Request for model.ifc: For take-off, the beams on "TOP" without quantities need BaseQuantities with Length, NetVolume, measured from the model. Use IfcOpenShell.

First a look at what the model holds.

```python
import ifcopenshell
import ifcopenshell.util.element
import ifcopenshell.util.unit

model = ifcopenshell.open("model.ifc")
print(model.schema)
for unit_type in ("LENGTHUNIT", "AREAUNIT", "VOLUMEUNIT"):
    print(unit_type, ifcopenshell.util.unit.calculate_unit_scale(model, unit_type))
storey = next(s for s in model.by_type("IfcBuildingStorey") if s.Name == "TOP")
beams = [e for e in ifcopenshell.util.element.get_decomposition(storey) if e.is_a("IfcBeam")]
for e in sorted(beams, key=lambda e: e.id()):
    print(e.id(), e.is_a(), e.Name, list(ifcopenshell.util.element.get_psets(e, qtos_only=True)), sep=" | ")
```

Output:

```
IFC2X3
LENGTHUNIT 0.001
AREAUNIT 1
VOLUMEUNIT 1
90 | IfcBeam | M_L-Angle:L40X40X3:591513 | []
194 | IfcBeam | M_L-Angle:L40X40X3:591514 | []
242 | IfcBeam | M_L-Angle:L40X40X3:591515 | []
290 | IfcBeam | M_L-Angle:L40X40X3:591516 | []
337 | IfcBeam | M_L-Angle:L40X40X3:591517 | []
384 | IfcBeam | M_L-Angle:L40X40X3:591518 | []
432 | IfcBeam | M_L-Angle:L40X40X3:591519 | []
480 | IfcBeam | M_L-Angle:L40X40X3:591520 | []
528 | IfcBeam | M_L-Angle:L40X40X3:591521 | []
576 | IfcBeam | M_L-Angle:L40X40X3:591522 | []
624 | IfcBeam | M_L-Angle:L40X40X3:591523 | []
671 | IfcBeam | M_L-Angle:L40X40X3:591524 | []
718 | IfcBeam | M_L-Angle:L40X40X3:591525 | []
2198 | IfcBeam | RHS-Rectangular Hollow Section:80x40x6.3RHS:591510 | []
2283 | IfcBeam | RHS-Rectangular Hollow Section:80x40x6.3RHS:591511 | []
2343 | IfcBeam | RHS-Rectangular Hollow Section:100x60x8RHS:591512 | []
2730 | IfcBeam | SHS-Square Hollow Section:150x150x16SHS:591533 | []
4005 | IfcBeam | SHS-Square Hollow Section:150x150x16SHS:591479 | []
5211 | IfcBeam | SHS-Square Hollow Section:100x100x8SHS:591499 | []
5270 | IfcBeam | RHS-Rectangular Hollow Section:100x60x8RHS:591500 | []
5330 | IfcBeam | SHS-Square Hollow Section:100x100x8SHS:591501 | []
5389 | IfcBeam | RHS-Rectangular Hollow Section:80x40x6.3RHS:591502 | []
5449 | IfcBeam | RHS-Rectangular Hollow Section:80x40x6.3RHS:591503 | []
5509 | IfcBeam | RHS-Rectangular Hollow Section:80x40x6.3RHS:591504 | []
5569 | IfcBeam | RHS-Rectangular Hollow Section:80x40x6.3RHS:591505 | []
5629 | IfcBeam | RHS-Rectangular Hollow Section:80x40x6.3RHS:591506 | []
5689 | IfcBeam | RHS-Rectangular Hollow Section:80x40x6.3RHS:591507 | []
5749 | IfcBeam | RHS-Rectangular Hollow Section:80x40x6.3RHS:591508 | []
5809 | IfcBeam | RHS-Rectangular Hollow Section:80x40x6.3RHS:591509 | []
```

```python
import ifcopenshell
import ifcopenshell.api.pset
import ifcopenshell.geom
import ifcopenshell.util.element
import ifcopenshell.util.shape
import ifcopenshell.util.unit

model = ifcopenshell.open("model.ifc")
unit_scale = ifcopenshell.util.unit.calculate_unit_scale(model)
volume_scale = ifcopenshell.util.unit.calculate_unit_scale(model, "VOLUMEUNIT")
settings = ifcopenshell.geom.settings()

storey = next(s for s in model.by_type("IfcBuildingStorey") if s.Name == "TOP")
beams = [e for e in ifcopenshell.util.element.get_decomposition(storey) if e.is_a("IfcBeam")]

for e in sorted(beams, key=lambda e: e.id()):
    if ifcopenshell.util.element.get_psets(e, qtos_only=True, should_inherit=False):
        continue
    # Geometry comes back in metres, in the element's own axes.
    shape = ifcopenshell.geom.create_shape(settings, e)
    values = {
        "Length": ifcopenshell.util.shape.get_max_xyz(shape.geometry) / unit_scale,
        "NetVolume": ifcopenshell.util.shape.get_volume(shape.geometry) / volume_scale,
    }
    qto = ifcopenshell.api.pset.add_qto(model, product=e, name="BaseQuantities")
    ifcopenshell.api.pset.edit_qto(model, qto=qto, properties=values)
    print(e.id(), {k: round(v, 3) for k, v in values.items()})

model.write("model_updated.ifc")
```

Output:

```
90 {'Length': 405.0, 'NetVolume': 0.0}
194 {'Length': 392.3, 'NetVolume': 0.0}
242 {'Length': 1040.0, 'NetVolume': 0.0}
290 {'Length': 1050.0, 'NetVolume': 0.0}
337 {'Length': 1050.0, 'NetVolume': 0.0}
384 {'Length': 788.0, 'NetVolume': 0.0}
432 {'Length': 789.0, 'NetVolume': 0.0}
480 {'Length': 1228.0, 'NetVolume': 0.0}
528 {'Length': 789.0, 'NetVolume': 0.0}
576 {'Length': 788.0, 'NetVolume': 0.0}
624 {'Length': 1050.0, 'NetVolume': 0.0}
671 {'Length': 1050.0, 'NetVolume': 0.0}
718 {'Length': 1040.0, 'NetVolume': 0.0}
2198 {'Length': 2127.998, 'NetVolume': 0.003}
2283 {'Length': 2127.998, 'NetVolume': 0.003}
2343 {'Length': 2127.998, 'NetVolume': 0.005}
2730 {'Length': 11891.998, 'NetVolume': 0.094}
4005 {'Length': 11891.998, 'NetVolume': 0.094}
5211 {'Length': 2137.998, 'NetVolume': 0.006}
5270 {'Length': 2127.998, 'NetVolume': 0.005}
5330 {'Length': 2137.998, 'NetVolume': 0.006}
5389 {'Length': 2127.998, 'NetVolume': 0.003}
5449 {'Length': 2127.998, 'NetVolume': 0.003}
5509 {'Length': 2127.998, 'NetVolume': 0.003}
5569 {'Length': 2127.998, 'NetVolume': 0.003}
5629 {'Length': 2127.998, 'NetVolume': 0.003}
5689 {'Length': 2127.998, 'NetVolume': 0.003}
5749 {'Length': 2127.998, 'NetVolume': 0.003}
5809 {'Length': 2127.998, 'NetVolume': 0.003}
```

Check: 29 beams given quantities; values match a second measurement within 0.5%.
